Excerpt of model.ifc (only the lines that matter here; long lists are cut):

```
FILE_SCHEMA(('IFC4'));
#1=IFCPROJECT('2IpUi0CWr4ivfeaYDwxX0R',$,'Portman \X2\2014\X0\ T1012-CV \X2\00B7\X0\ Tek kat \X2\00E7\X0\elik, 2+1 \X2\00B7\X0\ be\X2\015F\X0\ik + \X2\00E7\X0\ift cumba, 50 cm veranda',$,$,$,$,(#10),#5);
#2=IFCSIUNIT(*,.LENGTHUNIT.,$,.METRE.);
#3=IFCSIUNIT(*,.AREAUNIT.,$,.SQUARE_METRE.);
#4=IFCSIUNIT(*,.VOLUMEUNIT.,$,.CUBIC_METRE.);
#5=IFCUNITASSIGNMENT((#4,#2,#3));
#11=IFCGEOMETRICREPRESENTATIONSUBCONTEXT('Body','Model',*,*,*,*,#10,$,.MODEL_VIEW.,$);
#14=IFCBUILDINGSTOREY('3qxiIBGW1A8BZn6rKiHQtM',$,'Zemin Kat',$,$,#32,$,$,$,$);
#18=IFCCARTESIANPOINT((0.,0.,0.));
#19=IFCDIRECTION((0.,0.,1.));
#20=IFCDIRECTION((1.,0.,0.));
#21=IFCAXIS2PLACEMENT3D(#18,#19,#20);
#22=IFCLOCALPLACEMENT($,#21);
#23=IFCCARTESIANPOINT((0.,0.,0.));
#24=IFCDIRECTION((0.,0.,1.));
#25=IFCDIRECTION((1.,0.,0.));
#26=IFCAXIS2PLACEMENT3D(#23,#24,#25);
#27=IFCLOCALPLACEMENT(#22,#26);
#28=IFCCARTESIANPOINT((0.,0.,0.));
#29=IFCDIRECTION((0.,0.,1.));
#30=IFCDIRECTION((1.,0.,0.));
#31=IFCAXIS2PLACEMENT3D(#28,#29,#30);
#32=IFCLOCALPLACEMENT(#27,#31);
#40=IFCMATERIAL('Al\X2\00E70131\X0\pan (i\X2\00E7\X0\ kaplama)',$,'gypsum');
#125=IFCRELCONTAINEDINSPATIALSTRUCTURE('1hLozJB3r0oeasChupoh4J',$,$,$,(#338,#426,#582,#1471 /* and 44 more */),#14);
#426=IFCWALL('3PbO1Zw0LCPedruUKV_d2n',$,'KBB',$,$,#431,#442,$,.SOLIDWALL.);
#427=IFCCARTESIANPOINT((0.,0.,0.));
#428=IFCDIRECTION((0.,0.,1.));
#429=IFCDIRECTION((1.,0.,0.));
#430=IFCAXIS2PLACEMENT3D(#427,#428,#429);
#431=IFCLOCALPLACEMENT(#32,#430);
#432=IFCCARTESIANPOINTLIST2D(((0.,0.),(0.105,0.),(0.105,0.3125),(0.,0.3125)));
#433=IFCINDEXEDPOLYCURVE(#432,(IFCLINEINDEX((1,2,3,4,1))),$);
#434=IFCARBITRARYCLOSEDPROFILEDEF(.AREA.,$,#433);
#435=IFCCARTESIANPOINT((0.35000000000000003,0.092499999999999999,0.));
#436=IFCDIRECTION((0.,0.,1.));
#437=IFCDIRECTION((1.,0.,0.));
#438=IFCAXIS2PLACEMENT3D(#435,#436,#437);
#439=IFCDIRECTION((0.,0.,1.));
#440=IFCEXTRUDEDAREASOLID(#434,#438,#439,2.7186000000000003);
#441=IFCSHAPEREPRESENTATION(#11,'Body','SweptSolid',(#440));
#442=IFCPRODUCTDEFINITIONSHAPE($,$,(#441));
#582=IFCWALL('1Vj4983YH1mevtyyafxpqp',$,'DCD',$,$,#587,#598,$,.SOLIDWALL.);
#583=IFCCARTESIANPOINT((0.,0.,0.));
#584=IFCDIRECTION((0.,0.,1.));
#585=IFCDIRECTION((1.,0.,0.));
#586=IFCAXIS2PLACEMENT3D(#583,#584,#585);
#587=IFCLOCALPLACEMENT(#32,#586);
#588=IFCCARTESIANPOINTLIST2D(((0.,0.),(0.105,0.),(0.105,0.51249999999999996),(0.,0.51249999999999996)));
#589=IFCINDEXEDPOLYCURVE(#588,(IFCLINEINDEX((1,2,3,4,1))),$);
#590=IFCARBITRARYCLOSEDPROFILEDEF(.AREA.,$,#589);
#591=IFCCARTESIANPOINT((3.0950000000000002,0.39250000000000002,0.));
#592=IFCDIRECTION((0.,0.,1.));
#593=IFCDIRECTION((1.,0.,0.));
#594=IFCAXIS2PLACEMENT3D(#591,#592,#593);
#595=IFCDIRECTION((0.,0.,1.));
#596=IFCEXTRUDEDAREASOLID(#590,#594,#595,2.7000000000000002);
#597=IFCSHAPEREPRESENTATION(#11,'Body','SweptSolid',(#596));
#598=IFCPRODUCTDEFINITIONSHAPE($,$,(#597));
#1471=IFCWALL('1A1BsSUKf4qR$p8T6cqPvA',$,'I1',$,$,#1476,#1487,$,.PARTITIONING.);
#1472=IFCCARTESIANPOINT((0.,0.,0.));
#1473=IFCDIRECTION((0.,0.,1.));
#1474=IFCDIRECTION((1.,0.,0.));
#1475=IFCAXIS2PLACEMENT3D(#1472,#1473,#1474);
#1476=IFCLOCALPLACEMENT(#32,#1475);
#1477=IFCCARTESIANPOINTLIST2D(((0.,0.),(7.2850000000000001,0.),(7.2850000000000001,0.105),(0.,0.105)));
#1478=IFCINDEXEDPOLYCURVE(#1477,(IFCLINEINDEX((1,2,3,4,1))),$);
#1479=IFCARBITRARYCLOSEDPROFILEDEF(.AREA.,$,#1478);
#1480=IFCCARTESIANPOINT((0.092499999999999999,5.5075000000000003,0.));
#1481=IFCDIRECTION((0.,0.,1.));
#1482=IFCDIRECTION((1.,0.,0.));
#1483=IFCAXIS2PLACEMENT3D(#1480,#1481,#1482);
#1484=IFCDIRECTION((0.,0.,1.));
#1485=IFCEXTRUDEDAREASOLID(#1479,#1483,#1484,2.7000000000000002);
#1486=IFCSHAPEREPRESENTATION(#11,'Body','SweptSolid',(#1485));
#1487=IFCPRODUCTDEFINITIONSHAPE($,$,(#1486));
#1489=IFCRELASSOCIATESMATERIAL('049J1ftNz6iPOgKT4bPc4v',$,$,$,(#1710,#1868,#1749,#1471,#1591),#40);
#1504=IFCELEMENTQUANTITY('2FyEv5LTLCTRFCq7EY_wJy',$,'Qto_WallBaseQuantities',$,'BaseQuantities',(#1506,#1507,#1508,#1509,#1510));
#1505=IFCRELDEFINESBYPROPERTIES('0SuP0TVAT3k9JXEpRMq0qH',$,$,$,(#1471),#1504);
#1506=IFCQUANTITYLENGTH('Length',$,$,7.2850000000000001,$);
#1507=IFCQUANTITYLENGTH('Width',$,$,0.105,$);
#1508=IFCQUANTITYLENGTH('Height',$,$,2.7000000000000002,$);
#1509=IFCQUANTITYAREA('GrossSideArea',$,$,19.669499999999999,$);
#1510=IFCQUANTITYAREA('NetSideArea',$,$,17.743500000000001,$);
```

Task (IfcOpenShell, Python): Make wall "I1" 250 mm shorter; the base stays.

```python
import ifcopenshell
import ifcopenshell.api.pset
import ifcopenshell.geom
import ifcopenshell.util.element
import ifcopenshell.util.representation
import ifcopenshell.util.shape
import ifcopenshell.util.unit

model = ifcopenshell.open("model.ifc")
unit_scale = ifcopenshell.util.unit.calculate_unit_scale(model)
area_scale = ifcopenshell.util.unit.calculate_unit_scale(model, "AREAUNIT")
settings = ifcopenshell.geom.settings()


def volume(element):
    """Net volume in cubic metres, openings subtracted."""
    shape = ifcopenshell.geom.create_shape(settings, element)
    return ifcopenshell.util.shape.get_volume(shape.geometry)


wall = model.by_guid("1A1BsSUKf4qR$p8T6cqPvA")
before = volume(wall)

body = ifcopenshell.util.representation.get_representation(wall, "Model", "Body")
solid = body.Items[0]
old_height = solid.Depth
solid.Depth -= 0.25 / unit_scale
after = volume(wall)
thickness = 0.105  # wall thickness in metres

# Update the stored height, areas and volumes.
qto = model.by_id(ifcopenshell.util.element.get_pset(wall, "Qto_WallBaseQuantities", should_inherit=False)["id"])
ifcopenshell.api.pset.edit_qto(model, qto=qto, properties={
    "Height": solid.Depth,
    "GrossSideArea": ifcopenshell.util.element.get_pset(wall, "Qto_WallBaseQuantities", "GrossSideArea") * solid.Depth / old_height,
    "NetSideArea": after / thickness / area_scale,
})

print(f"height {old_height:g} -> {solid.Depth:g}, volume {before:.3f} -> {after:.3f} m3")

model.write("model_updated.ifc")
```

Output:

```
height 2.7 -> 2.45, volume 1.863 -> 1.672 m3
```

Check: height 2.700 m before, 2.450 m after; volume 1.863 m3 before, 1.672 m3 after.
